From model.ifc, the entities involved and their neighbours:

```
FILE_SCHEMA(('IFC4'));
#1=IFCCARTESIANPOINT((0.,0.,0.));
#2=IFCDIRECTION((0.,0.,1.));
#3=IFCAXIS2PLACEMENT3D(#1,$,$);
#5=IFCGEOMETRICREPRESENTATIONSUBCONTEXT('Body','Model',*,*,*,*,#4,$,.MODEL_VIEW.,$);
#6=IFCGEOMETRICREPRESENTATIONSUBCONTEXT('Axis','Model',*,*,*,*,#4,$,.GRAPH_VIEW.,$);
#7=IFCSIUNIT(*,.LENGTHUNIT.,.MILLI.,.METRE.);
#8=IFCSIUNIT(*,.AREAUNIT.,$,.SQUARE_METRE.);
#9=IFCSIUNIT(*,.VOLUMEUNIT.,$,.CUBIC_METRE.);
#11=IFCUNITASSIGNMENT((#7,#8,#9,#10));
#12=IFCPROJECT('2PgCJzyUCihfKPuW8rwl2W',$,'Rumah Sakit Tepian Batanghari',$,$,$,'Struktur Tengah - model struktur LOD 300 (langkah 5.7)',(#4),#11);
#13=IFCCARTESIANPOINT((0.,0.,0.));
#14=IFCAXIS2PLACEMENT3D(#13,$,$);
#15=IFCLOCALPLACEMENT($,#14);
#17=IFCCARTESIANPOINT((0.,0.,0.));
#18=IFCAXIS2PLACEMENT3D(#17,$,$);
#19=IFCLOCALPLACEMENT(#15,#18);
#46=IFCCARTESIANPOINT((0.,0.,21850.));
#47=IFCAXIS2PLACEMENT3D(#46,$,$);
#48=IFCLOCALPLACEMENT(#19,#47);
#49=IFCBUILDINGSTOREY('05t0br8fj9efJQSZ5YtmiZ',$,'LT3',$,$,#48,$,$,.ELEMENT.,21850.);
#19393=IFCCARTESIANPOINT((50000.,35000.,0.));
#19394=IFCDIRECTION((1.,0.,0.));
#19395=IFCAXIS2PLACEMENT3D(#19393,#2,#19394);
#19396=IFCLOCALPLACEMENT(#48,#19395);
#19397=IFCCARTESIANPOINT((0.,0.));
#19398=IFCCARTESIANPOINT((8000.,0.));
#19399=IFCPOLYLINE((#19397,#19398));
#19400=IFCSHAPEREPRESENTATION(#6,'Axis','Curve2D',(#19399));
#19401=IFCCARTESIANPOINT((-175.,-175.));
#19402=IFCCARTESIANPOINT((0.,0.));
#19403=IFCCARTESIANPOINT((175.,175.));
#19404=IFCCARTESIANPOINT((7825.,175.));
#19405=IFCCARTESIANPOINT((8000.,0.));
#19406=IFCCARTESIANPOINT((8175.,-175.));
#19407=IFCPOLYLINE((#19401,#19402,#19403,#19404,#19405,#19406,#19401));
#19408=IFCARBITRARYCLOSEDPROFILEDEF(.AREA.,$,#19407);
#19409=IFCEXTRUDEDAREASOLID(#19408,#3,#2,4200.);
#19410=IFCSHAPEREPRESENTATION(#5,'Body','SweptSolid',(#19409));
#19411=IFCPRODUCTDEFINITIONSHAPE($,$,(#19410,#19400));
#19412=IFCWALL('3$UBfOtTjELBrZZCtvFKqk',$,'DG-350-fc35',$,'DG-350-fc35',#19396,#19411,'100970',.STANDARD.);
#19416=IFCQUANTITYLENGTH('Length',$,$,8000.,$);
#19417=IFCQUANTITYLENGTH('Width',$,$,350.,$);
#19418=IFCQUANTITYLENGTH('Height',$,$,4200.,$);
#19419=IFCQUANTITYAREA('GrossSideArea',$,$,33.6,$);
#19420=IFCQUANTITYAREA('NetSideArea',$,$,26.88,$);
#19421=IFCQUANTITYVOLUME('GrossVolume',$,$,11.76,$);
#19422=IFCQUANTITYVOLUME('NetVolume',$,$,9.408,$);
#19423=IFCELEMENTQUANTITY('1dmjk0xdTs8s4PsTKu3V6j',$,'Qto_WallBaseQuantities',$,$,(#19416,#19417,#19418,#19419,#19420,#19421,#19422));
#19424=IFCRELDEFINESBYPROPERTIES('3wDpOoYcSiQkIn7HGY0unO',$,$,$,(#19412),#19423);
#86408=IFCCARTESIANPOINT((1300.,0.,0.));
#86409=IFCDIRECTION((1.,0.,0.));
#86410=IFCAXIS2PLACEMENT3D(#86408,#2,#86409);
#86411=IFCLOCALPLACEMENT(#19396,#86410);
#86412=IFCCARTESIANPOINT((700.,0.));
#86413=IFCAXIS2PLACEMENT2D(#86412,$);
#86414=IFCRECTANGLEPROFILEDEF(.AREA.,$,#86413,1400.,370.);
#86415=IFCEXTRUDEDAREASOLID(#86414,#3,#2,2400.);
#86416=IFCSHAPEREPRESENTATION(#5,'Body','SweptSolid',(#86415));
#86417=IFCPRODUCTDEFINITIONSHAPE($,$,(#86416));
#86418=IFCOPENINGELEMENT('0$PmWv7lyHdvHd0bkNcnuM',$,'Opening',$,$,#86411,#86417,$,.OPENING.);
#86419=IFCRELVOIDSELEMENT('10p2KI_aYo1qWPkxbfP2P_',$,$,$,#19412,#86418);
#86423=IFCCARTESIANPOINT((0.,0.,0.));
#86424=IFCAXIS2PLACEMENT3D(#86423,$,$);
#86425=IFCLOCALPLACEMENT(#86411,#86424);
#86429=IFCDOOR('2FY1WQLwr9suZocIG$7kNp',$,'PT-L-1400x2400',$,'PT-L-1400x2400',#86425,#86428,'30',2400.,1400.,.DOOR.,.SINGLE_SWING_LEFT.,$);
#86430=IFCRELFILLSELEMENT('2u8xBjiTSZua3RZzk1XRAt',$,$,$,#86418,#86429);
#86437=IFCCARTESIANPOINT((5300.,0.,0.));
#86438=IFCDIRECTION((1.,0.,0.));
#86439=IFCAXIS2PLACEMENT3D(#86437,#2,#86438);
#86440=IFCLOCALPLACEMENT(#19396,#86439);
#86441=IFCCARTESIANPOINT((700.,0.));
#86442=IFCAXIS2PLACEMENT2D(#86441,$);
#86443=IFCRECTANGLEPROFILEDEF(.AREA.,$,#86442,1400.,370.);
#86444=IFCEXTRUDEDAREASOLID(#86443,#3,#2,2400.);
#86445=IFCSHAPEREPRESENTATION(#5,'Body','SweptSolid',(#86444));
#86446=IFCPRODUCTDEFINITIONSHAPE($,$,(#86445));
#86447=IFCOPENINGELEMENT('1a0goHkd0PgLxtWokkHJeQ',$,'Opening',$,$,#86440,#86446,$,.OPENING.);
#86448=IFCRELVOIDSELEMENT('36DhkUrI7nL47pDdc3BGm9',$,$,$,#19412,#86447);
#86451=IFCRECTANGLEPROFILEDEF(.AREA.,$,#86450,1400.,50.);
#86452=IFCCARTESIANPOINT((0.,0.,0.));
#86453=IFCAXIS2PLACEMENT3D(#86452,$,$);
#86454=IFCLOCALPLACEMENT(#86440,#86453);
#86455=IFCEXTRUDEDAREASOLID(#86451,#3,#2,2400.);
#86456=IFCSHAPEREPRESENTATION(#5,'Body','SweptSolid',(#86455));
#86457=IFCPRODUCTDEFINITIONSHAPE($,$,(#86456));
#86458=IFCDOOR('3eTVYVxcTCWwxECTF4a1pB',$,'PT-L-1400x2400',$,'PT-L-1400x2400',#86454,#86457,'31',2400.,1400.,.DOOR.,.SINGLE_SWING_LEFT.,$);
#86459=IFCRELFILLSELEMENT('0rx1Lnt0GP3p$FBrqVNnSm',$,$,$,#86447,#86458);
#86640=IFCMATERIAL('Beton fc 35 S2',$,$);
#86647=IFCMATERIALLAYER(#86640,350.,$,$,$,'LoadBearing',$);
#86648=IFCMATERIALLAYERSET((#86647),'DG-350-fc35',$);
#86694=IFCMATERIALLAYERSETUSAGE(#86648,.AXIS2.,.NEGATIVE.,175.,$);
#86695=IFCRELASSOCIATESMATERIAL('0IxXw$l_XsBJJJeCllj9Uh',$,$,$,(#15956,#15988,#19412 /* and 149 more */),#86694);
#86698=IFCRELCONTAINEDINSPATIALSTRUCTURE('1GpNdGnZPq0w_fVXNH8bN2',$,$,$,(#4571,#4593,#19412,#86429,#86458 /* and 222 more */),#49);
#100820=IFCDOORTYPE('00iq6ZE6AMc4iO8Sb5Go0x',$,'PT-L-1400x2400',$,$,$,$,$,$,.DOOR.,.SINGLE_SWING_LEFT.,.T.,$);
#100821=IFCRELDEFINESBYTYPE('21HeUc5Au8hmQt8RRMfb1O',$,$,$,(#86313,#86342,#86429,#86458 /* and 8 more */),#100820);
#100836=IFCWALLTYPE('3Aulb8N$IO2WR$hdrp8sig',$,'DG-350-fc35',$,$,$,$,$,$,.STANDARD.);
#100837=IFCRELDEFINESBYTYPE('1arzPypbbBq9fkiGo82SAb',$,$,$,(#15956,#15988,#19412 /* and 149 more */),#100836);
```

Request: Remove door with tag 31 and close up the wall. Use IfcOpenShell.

```python
import ifcopenshell
import ifcopenshell.api.feature
import ifcopenshell.api.pset
import ifcopenshell.api.root
import ifcopenshell.geom
import ifcopenshell.util.element
import ifcopenshell.util.shape
import ifcopenshell.util.unit

model = ifcopenshell.open("model.ifc")
area_scale = ifcopenshell.util.unit.calculate_unit_scale(model, "AREAUNIT")
volume_scale = ifcopenshell.util.unit.calculate_unit_scale(model, "VOLUMEUNIT")
settings = ifcopenshell.geom.settings()


def volume(element):
    """Net volume in cubic metres, openings subtracted."""
    shape = ifcopenshell.geom.create_shape(settings, element)
    return ifcopenshell.util.shape.get_volume(shape.geometry)


door = model.by_guid("3eTVYVxcTCWwxECTF4a1pB")
opening = door.FillsVoids[0].RelatingOpeningElement
wall = opening.VoidsElements[0].RelatingBuildingElement
before = volume(wall)

ifcopenshell.api.root.remove_product(model, product=door)
ifcopenshell.api.feature.remove_feature(model, feature=opening)

after = volume(wall)
thickness = 0.35  # wall thickness in metres

# Update the wall's stored quantities.
qto = model.by_id(ifcopenshell.util.element.get_pset(wall, "Qto_WallBaseQuantities", should_inherit=False)["id"])
ifcopenshell.api.pset.edit_qto(model, qto=qto, properties={
    "NetSideArea": after / thickness / area_scale,
    "NetVolume": after / volume_scale,
})

print(f"wall volume {before:.3f} -> {after:.3f} m3")

model.write("model-out.ifc")
```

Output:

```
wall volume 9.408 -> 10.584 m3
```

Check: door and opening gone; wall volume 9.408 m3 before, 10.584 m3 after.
